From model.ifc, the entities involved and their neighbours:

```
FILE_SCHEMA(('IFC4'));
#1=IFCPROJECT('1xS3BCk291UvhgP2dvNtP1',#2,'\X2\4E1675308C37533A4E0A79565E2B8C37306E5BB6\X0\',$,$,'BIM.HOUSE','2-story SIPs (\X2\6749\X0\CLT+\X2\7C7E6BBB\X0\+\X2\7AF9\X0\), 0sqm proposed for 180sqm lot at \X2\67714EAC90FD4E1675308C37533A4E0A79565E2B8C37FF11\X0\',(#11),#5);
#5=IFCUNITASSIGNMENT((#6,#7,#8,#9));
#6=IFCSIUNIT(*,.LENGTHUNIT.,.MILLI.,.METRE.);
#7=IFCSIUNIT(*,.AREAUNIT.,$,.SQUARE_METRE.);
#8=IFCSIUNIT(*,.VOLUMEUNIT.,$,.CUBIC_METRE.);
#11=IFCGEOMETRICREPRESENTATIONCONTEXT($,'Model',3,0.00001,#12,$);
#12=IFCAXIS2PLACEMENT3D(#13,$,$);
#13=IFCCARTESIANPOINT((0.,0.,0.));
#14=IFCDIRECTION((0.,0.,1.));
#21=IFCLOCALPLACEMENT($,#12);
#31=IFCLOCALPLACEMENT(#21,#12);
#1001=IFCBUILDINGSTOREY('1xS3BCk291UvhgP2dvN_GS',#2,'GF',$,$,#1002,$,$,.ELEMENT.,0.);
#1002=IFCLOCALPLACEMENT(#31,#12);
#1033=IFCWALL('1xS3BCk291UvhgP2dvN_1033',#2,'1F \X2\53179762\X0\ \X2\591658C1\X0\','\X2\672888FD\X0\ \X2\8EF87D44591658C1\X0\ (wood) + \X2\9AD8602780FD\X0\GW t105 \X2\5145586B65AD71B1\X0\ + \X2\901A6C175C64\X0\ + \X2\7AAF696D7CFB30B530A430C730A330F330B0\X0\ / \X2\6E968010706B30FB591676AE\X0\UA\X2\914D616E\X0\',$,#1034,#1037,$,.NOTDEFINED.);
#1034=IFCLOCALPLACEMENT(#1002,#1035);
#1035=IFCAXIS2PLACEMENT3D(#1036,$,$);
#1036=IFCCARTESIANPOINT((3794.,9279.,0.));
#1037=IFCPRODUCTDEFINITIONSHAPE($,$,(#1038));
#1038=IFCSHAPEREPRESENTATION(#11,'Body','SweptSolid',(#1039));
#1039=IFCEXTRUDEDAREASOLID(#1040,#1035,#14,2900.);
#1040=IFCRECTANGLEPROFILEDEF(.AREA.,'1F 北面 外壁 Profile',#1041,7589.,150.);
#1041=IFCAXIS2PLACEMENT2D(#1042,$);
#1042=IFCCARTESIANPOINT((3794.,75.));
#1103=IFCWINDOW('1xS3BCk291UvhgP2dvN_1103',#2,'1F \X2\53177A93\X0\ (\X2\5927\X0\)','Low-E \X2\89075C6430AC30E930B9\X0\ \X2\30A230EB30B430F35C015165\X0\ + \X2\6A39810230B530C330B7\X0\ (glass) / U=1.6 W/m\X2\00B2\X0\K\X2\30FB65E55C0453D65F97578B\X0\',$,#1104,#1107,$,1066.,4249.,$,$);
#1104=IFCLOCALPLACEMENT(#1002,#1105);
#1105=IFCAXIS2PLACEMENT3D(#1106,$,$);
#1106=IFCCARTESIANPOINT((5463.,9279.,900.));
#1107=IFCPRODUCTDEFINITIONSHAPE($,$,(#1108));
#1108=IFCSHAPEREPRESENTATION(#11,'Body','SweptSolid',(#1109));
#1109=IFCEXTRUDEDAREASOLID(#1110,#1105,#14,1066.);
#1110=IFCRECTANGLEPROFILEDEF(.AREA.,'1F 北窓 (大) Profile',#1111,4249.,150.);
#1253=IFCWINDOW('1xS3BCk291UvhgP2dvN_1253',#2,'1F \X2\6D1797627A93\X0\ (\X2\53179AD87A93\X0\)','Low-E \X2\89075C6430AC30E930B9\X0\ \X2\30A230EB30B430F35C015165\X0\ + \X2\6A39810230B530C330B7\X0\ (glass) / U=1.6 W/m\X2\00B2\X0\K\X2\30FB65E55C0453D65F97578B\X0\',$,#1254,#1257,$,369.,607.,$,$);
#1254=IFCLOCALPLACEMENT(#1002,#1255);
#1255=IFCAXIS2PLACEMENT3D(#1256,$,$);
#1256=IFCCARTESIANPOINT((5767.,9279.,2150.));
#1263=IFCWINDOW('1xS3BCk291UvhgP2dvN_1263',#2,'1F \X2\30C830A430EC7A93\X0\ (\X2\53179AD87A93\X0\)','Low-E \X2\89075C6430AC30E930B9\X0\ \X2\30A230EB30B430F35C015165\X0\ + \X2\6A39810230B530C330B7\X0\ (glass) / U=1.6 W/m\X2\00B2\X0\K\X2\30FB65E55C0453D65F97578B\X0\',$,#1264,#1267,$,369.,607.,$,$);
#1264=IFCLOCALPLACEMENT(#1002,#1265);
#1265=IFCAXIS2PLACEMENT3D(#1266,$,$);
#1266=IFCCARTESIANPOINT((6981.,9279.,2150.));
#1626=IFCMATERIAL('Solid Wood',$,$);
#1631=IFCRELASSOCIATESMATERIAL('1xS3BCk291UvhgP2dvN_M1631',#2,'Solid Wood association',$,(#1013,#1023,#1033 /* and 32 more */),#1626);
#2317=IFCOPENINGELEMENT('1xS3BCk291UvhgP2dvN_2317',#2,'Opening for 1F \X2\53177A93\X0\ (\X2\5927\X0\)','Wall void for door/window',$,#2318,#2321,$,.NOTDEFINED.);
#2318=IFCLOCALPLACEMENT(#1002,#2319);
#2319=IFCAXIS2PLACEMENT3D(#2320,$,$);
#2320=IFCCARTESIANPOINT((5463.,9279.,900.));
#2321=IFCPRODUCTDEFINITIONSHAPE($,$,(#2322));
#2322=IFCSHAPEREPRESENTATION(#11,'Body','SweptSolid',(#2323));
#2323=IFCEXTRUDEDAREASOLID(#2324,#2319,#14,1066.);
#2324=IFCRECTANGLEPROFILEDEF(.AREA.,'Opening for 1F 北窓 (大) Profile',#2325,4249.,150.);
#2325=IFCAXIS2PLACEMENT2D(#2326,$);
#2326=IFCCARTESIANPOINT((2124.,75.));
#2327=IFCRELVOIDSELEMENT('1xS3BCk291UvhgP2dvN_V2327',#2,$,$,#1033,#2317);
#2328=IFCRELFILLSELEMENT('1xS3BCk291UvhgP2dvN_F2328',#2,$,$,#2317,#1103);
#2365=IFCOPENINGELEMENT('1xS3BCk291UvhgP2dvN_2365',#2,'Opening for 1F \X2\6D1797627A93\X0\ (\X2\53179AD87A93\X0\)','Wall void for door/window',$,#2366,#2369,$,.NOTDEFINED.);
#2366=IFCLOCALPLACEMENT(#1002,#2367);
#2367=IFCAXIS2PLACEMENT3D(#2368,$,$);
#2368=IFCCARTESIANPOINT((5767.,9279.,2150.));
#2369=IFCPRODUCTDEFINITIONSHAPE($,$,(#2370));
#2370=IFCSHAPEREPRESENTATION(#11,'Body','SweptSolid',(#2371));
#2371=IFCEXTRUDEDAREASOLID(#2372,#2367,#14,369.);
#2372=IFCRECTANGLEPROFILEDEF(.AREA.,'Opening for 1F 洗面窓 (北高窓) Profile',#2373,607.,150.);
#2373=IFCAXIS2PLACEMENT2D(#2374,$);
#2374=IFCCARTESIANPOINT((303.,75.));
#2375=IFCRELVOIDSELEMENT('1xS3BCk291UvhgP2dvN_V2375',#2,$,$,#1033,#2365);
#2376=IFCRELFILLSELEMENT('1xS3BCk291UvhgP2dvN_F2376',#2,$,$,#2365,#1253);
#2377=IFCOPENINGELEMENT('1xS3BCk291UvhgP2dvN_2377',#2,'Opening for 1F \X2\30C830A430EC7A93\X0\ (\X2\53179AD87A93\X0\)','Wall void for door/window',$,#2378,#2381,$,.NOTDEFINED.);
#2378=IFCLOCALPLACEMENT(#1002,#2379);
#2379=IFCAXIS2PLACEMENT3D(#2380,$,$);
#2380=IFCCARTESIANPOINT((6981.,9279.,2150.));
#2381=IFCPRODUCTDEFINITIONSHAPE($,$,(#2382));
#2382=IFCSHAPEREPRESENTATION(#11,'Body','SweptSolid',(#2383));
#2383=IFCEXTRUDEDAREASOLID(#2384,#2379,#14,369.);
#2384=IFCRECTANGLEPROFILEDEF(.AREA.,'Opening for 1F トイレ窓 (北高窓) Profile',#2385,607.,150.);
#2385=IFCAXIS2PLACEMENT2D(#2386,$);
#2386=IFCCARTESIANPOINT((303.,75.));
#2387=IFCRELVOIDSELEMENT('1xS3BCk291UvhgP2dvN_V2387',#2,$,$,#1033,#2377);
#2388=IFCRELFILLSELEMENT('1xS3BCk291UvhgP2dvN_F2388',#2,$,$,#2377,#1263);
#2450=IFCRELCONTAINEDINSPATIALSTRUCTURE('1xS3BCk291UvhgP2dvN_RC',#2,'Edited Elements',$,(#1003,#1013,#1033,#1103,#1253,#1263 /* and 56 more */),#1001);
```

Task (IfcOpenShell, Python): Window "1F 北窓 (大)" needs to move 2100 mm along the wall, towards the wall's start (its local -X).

```python
import ifcopenshell
import ifcopenshell.api.geometry
import ifcopenshell.util.placement
import ifcopenshell.util.unit

model = ifcopenshell.open("model.ifc")
unit_scale = ifcopenshell.util.unit.calculate_unit_scale(model)

window = model.by_guid("1xS3BCk291UvhgP2dvN_1103")
opening = window.FillsVoids[0].RelatingOpeningElement
wall = opening.VoidsElements[0].RelatingBuildingElement

wall_matrix = ifcopenshell.util.placement.get_local_placement(wall.ObjectPlacement)
shift = wall_matrix[:3, 0] * -2.1 / unit_scale
before = ifcopenshell.util.placement.get_local_placement(window.ObjectPlacement)[:3, 3].copy()

# The window is not placed relative to its opening, so move both.
for product in (opening, window):
    matrix = ifcopenshell.util.placement.get_local_placement(product.ObjectPlacement)
    matrix[:3, 3] += shift
    ifcopenshell.api.geometry.edit_object_placement(model, product=product, matrix=matrix, is_si=False)

after = ifcopenshell.util.placement.get_local_placement(window.ObjectPlacement)[:3, 3]
print("window moved by", (after - before).round(3) + 0.0)

model.write("model-out.ifc")
```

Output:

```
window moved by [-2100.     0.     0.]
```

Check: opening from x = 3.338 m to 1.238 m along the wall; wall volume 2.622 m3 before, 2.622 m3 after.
